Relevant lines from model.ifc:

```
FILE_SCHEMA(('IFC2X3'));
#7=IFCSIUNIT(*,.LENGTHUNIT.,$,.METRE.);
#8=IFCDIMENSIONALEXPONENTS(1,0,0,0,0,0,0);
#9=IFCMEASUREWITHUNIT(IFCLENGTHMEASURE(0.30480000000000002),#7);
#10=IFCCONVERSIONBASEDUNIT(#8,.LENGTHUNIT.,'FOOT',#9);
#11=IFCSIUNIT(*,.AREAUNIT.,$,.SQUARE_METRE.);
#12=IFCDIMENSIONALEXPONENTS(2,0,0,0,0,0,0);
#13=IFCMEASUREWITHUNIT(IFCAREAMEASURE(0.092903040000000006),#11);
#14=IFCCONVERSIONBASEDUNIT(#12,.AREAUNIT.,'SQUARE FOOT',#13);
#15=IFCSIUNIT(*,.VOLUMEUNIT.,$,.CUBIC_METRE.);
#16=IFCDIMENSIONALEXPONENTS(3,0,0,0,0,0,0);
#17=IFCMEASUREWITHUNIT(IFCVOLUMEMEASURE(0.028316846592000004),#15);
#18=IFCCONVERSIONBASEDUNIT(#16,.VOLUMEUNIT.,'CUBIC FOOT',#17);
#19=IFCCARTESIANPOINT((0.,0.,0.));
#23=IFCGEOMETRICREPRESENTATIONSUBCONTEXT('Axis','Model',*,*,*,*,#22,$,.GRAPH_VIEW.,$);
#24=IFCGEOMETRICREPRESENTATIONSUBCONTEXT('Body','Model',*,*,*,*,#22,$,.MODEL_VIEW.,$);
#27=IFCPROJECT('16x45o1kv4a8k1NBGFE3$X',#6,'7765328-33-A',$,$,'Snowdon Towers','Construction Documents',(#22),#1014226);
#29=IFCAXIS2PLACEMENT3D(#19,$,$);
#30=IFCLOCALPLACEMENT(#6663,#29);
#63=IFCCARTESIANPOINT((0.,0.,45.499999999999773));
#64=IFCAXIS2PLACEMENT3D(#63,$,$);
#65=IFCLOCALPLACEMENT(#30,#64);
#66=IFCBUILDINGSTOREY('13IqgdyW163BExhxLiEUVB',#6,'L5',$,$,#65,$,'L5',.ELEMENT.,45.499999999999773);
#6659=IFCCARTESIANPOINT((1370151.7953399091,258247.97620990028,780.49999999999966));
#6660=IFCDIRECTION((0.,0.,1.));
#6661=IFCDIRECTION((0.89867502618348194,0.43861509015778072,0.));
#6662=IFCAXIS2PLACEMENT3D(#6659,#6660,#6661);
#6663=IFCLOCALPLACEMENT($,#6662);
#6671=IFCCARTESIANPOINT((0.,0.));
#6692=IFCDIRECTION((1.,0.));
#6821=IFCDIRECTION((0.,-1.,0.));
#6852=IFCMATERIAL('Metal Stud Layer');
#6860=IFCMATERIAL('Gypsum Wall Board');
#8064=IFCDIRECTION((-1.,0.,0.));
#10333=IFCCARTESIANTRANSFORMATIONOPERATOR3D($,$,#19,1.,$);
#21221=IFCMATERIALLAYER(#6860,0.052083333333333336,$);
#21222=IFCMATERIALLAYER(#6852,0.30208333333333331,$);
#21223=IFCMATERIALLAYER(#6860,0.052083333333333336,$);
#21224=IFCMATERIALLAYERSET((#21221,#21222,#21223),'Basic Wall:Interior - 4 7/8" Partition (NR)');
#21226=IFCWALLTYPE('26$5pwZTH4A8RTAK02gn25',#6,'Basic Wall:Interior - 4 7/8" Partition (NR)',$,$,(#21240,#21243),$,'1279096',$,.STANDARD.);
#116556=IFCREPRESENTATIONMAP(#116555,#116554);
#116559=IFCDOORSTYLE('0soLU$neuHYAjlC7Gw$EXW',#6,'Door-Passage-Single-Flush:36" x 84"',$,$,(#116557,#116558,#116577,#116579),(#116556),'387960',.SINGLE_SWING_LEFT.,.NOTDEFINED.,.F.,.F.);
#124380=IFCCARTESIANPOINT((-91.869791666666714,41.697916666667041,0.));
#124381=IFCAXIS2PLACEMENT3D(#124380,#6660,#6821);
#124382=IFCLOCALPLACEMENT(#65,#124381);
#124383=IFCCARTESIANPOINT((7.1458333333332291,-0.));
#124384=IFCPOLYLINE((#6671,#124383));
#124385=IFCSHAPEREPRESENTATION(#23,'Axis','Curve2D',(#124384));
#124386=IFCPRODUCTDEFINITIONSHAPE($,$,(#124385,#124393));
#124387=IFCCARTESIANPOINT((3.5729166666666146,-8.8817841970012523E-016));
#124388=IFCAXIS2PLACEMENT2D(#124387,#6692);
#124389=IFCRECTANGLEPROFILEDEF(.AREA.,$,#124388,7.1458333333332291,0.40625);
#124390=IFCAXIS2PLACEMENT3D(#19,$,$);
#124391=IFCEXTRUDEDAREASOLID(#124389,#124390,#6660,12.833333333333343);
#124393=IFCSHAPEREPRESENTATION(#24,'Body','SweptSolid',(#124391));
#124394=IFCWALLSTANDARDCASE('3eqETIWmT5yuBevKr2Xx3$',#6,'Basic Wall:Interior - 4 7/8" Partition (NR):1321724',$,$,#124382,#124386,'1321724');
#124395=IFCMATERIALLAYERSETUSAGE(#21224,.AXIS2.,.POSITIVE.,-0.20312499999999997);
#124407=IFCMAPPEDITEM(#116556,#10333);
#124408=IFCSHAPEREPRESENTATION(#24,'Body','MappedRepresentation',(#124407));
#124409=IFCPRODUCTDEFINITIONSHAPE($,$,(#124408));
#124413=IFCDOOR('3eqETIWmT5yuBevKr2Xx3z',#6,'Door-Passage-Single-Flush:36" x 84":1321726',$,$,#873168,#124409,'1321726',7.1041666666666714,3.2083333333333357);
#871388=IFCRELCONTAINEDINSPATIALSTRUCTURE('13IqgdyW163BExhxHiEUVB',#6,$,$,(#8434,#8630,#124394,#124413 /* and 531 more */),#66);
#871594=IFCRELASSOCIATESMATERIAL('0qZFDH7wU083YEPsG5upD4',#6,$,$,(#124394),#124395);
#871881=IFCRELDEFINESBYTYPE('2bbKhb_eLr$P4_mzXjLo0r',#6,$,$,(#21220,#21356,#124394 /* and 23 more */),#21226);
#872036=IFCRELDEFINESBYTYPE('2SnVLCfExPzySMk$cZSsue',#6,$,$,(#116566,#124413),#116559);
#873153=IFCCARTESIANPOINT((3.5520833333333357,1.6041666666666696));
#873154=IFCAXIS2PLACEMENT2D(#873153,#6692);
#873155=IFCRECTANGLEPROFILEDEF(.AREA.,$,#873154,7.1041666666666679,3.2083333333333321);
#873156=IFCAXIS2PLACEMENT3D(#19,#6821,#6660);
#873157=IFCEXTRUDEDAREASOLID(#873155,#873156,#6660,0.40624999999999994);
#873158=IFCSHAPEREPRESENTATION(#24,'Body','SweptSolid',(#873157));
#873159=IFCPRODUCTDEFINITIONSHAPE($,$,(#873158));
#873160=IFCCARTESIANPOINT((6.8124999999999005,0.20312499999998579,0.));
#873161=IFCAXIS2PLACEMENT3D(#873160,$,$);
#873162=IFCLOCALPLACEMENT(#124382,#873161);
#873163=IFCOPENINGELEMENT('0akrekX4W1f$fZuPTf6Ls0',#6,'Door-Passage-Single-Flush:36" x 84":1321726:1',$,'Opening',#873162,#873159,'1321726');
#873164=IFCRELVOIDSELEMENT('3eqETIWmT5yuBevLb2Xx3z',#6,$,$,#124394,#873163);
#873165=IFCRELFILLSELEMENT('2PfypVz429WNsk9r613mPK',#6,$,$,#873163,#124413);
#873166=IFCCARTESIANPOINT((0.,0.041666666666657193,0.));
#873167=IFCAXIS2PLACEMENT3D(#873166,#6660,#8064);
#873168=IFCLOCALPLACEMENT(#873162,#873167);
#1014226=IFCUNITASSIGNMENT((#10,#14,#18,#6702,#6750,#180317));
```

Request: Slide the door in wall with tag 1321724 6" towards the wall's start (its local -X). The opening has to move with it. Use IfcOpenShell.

```python
import ifcopenshell
import ifcopenshell.api.geometry
import ifcopenshell.util.placement
import ifcopenshell.util.unit

model = ifcopenshell.open("model.ifc")
unit_scale = ifcopenshell.util.unit.calculate_unit_scale(model)

door = model.by_id(124413)
opening = door.FillsVoids[0].RelatingOpeningElement
wall = opening.VoidsElements[0].RelatingBuildingElement

wall_matrix = ifcopenshell.util.placement.get_local_placement(wall.ObjectPlacement)
shift = wall_matrix[:3, 0] * -6 * 0.0254 / unit_scale
before = ifcopenshell.util.placement.get_local_placement(door.ObjectPlacement)[:3, 3].copy()

# The door is placed relative to its opening, so it follows when the opening moves.
matrix = ifcopenshell.util.placement.get_local_placement(opening.ObjectPlacement)
matrix[:3, 3] += shift
ifcopenshell.api.geometry.edit_object_placement(
    model, product=opening, matrix=matrix, is_si=False, should_transform_children=True
)

after = ifcopenshell.util.placement.get_local_placement(door.ObjectPlacement)[:3, 3]
print("door moved by", (after - before).round(3) + 0.0)

model.write("model_v2.ifc")
```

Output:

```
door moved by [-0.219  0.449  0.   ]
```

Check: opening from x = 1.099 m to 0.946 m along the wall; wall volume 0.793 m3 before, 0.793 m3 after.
